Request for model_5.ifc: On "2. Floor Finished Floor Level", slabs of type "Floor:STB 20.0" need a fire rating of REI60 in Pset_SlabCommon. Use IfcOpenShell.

First a look at what the model holds.

```python
import ifcopenshell
import ifcopenshell.util.element

model = ifcopenshell.open("model_5.ifc")
print(model.schema)
storey = next(s for s in model.by_type("IfcBuildingStorey") if s.Name == "2. Floor Finished Floor Level")
slabs = [e for e in ifcopenshell.util.element.get_decomposition(storey) if e.is_a("IfcSlab")]
seen = {}
for e in slabs:
    element_type = ifcopenshell.util.element.get_type(e)
    key = (element_type.Name if element_type != e and element_type else None, ifcopenshell.util.element.get_pset(e, "Pset_SlabCommon", "FireRating"))
    seen[key] = seen.get(key, 0) + 1
for (name, value), count in sorted(seen.items(), key=str):
    print(count, "x", name, "|", value)
```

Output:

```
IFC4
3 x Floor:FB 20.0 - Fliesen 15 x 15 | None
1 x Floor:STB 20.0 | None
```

```python
import ifcopenshell
import ifcopenshell.api.pset
import ifcopenshell.util.element

model = ifcopenshell.open("model_5.ifc")

storey = next(s for s in model.by_type("IfcBuildingStorey") if s.Name == "2. Floor Finished Floor Level")
slabs = [e for e in ifcopenshell.util.element.get_decomposition(storey) if e.is_a("IfcSlab")]

count = 0
for e in slabs:
    element_type = ifcopenshell.util.element.get_type(e)
    if element_type in (None, e) or element_type.Name != "Floor:STB 20.0":
        continue
    # add_pset returns the element's existing set when there is one.
    pset = ifcopenshell.api.pset.add_pset(model, product=e, name="Pset_SlabCommon")
    ifcopenshell.api.pset.edit_pset(model, pset=pset, properties={"FireRating": "REI60"})
    count += 1

print(count, "slabs updated")

model.write("model_5_v2.ifc")
```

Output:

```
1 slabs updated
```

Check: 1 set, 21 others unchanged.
